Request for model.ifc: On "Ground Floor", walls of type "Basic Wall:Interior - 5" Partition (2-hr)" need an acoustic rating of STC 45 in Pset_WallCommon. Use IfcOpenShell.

First a look at what the model holds.

```python
import ifcopenshell
import ifcopenshell.util.element

model = ifcopenshell.open("model.ifc")
print(model.schema)
storey = next(s for s in model.by_type("IfcBuildingStorey") if s.Name == "Ground Floor")
walls = [e for e in ifcopenshell.util.element.get_decomposition(storey) if e.is_a("IfcWall")]
seen = {}
for e in walls:
    element_type = ifcopenshell.util.element.get_type(e)
    key = (element_type.Name if element_type != e and element_type else None, ifcopenshell.util.element.get_pset(e, "Pset_WallCommon", "AcousticRating"))
    seen[key] = seen.get(key, 0) + 1
for (name, value), count in sorted(seen.items(), key=str):
    print(count, "x", name, "|", value)
```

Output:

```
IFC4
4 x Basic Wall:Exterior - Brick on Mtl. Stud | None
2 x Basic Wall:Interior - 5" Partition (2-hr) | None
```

```python
import ifcopenshell
import ifcopenshell.api.pset
import ifcopenshell.util.element

model = ifcopenshell.open("model.ifc")

storey = next(s for s in model.by_type("IfcBuildingStorey") if s.Name == "Ground Floor")
walls = [e for e in ifcopenshell.util.element.get_decomposition(storey) if e.is_a("IfcWall")]

count = 0
for e in walls:
    element_type = ifcopenshell.util.element.get_type(e)
    if element_type in (None, e) or element_type.Name != 'Basic Wall:Interior - 5" Partition (2-hr)':
        continue
    # add_pset returns the element's existing set when there is one.
    pset = ifcopenshell.api.pset.add_pset(model, product=e, name="Pset_WallCommon")
    ifcopenshell.api.pset.edit_pset(model, pset=pset, properties={"AcousticRating": "STC 45"})
    count += 1

print(count, "walls updated")

model.write("model-out.ifc")
```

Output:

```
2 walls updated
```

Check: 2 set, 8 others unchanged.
